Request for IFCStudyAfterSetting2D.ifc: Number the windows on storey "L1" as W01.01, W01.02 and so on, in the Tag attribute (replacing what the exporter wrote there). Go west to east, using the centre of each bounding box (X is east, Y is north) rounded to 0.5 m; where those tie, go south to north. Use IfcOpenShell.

First a look at what the model holds.

```python
import ifcopenshell
import ifcopenshell.util.element
import ifcopenshell.util.placement

model = ifcopenshell.open("IFCStudyAfterSetting2D.ifc")
print(model.schema)
storey = next(s for s in model.by_type("IfcBuildingStorey") if s.Name == "L1")
windows = [e for e in ifcopenshell.util.element.get_decomposition(storey) if e.is_a("IfcWindow")]
for e in sorted(windows, key=lambda e: e.id()):
    origin = ifcopenshell.util.placement.get_local_placement(e.ObjectPlacement)[:3, 3]
    print(e.id(), e.Tag, e.Name, origin.round(2) + 0.0, sep=" | ")
```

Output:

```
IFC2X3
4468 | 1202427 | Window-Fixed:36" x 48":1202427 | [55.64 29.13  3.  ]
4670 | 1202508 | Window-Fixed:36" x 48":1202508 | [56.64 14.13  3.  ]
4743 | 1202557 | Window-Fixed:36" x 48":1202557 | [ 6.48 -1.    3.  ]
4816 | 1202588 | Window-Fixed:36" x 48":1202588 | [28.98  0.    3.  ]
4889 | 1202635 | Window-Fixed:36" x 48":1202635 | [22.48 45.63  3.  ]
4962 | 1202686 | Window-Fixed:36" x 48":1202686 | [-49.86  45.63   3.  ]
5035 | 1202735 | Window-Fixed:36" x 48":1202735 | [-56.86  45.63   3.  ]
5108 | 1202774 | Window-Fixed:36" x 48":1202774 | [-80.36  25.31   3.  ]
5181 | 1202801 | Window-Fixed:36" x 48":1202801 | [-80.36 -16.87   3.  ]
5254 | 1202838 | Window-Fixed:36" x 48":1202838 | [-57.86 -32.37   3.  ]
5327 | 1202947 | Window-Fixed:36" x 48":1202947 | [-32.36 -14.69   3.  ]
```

```python
import ifcopenshell
import ifcopenshell.geom
import ifcopenshell.util.element
import ifcopenshell.util.shape

model = ifcopenshell.open("IFCStudyAfterSetting2D.ifc")
settings = ifcopenshell.geom.settings()
settings.set("use-world-coords", True)


def centre(element):
    shape = ifcopenshell.geom.create_shape(settings, element)
    return ifcopenshell.util.shape.get_bbox_centroid(shape.geometry)


storey = next(s for s in model.by_type("IfcBuildingStorey") if s.Name == "L1")
windows = [e for e in ifcopenshell.util.element.get_decomposition(storey) if e.is_a("IfcWindow")]

# Insertion points can sit at a corner or the storey origin, so sort by the geometry (in metres).
centres = {e: centre(e) for e in windows}
windows.sort(key=lambda e: (round(centres[e][0] / 0.5), centres[e][1]))

for i, e in enumerate(windows, start=1):
    number = f"W01.{i:02d}"
    e.Tag = number
    print(e.id(), number)

model.write("IFCStudyAfterSetting2D_updated.ifc")
```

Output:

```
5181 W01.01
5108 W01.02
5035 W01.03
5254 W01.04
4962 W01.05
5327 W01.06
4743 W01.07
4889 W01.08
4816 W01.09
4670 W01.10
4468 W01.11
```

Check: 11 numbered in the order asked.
